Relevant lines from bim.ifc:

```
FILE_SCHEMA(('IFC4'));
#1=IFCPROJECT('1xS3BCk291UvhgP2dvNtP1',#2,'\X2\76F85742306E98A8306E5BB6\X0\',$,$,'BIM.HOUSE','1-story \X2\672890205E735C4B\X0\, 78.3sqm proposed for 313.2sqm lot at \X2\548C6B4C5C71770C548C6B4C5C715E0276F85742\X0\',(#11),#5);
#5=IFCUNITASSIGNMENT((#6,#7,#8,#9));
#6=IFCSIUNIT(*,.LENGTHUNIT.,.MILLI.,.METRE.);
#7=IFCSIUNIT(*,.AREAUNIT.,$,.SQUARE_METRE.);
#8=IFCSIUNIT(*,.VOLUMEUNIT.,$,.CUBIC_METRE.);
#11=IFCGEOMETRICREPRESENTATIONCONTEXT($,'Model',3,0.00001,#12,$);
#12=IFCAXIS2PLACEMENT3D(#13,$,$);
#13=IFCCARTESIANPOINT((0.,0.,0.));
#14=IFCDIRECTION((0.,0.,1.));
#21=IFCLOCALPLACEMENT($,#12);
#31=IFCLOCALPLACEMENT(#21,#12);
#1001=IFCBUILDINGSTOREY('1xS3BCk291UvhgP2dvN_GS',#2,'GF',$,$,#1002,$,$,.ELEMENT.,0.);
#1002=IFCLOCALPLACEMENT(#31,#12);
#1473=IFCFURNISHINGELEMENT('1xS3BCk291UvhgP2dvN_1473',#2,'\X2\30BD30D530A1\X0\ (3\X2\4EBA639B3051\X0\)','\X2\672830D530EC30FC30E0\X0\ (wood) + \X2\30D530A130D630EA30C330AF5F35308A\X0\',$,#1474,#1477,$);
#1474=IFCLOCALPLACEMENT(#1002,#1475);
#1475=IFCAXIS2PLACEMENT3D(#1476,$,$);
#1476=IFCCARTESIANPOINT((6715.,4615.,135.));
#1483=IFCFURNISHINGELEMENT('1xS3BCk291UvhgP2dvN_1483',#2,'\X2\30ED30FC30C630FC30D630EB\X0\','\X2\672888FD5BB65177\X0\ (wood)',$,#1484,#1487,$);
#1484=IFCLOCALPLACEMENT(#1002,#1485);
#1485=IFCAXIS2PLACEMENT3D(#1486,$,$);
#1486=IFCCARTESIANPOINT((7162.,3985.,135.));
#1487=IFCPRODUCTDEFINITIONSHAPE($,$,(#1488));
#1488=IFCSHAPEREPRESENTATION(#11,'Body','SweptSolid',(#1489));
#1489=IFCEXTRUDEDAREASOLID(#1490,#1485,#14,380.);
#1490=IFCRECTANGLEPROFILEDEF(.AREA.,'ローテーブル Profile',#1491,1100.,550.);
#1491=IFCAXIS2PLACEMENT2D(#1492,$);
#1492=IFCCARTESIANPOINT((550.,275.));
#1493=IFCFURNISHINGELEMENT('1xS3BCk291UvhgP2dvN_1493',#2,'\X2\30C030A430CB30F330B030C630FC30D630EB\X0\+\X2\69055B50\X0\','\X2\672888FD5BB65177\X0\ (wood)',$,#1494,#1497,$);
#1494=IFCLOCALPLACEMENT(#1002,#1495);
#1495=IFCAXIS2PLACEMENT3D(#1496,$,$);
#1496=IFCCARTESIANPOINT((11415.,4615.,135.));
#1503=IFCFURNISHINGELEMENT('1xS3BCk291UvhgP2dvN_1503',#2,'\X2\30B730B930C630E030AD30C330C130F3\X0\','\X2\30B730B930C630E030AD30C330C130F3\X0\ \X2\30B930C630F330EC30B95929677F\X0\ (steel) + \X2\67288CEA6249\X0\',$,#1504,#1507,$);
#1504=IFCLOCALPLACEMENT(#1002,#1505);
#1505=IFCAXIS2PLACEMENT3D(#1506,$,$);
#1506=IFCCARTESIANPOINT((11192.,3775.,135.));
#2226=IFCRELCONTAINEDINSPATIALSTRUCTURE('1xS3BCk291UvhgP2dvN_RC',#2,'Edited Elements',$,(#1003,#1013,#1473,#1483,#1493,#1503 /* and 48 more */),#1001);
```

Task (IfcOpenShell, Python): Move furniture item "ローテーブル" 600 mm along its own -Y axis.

```python
import ifcopenshell
import ifcopenshell.api.geometry
import ifcopenshell.util.placement
import ifcopenshell.util.unit

model = ifcopenshell.open("bim.ifc")
unit_scale = ifcopenshell.util.unit.calculate_unit_scale(model)

item = model.by_guid("1xS3BCk291UvhgP2dvN_1483")
matrix = ifcopenshell.util.placement.get_local_placement(item.ObjectPlacement)
matrix[:3, 3] -= matrix[:3, 1] * 0.6 / unit_scale
ifcopenshell.api.geometry.edit_object_placement(model, product=item, matrix=matrix, is_si=False)

print(ifcopenshell.util.placement.get_local_placement(item.ObjectPlacement).round(3) + 0.0)

model.write("bim_v2.ifc")
```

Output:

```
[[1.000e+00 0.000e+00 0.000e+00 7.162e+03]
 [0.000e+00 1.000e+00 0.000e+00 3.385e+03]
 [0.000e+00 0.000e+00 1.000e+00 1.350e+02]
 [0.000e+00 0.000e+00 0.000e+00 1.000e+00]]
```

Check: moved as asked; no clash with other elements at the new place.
